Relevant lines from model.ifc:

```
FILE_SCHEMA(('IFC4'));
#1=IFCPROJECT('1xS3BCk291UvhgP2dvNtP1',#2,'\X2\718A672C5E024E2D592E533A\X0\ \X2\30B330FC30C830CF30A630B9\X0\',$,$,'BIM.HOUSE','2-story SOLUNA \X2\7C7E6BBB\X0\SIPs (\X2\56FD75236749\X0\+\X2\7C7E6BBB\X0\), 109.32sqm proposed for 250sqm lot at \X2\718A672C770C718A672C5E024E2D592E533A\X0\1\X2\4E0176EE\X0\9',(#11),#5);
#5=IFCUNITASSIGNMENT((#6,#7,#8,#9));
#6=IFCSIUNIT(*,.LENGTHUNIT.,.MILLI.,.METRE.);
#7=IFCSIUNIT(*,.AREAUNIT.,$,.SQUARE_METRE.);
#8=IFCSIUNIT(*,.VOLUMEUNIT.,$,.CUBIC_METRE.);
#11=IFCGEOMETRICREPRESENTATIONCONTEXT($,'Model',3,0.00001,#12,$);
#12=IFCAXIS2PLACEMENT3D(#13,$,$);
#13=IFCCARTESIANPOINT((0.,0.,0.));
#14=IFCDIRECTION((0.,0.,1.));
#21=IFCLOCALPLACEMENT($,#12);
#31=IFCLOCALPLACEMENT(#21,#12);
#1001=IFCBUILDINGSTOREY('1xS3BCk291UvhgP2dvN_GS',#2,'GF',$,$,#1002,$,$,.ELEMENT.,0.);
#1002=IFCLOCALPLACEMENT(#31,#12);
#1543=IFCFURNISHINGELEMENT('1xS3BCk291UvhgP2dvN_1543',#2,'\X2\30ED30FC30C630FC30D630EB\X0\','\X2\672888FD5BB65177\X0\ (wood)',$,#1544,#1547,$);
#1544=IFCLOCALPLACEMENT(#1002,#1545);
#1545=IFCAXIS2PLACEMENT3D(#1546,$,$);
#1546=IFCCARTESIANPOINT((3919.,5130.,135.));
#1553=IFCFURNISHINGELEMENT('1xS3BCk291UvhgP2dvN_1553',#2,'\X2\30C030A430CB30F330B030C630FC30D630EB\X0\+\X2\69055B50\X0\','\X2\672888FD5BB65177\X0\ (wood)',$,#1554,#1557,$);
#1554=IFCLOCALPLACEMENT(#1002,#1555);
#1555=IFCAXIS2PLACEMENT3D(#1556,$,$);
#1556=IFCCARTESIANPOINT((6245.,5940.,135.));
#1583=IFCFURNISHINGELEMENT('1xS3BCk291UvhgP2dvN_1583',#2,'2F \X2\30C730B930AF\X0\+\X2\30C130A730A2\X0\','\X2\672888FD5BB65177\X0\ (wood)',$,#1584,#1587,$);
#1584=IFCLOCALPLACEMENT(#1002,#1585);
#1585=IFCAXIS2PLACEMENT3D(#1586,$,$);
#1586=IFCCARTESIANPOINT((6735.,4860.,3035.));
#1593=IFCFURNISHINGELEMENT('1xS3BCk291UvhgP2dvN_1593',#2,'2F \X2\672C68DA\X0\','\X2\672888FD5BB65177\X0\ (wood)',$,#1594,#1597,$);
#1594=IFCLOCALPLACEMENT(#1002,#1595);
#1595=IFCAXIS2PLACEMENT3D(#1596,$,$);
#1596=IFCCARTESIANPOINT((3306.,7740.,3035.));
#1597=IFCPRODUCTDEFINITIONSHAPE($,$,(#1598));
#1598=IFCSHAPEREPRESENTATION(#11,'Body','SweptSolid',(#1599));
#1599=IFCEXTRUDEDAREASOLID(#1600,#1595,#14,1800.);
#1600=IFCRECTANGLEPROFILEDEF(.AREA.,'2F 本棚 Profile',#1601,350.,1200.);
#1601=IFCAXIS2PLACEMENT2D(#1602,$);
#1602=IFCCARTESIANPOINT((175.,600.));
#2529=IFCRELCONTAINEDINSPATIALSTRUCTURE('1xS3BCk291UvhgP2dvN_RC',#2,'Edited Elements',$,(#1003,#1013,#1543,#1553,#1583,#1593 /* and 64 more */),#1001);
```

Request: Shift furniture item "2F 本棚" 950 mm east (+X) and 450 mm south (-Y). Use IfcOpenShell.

```python
import ifcopenshell
import ifcopenshell.api.geometry
import ifcopenshell.util.placement
import ifcopenshell.util.unit

model = ifcopenshell.open("model.ifc")
unit_scale = ifcopenshell.util.unit.calculate_unit_scale(model)

item = model.by_guid("1xS3BCk291UvhgP2dvN_1593")
matrix = ifcopenshell.util.placement.get_local_placement(item.ObjectPlacement)
matrix[0, 3] += 0.95 / unit_scale
matrix[1, 3] -= 0.45 / unit_scale
ifcopenshell.api.geometry.edit_object_placement(model, product=item, matrix=matrix, is_si=False)

print(ifcopenshell.util.placement.get_local_placement(item.ObjectPlacement).round(3) + 0.0)

model.write("model_updated.ifc")
```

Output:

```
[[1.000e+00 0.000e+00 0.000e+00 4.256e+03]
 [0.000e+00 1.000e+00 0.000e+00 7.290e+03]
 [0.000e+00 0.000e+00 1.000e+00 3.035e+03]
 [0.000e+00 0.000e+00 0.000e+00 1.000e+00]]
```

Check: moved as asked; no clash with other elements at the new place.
